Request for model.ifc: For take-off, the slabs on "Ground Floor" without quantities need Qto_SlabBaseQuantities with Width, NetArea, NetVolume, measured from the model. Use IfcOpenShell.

First a look at what the model holds.

```python
import ifcopenshell
import ifcopenshell.util.element
import ifcopenshell.util.unit

model = ifcopenshell.open("model.ifc")
print(model.schema)
for unit_type in ("LENGTHUNIT", "AREAUNIT", "VOLUMEUNIT"):
    print(unit_type, ifcopenshell.util.unit.calculate_unit_scale(model, unit_type))
storey = next(s for s in model.by_type("IfcBuildingStorey") if s.Name == "Ground Floor")
slabs = [e for e in ifcopenshell.util.element.get_decomposition(storey) if e.is_a("IfcSlab")]
for e in sorted(slabs, key=lambda e: e.id()):
    print(e.id(), e.is_a(), e.Name, list(ifcopenshell.util.element.get_psets(e, qtos_only=True)), sep=" | ")
```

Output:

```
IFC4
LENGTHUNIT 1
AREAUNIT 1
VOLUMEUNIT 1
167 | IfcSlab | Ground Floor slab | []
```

```python
import ifcopenshell
import ifcopenshell.api.pset
import ifcopenshell.geom
import ifcopenshell.util.element
import ifcopenshell.util.shape
import ifcopenshell.util.unit

model = ifcopenshell.open("model.ifc")
unit_scale = ifcopenshell.util.unit.calculate_unit_scale(model)
area_scale = ifcopenshell.util.unit.calculate_unit_scale(model, "AREAUNIT")
volume_scale = ifcopenshell.util.unit.calculate_unit_scale(model, "VOLUMEUNIT")
settings = ifcopenshell.geom.settings()

storey = next(s for s in model.by_type("IfcBuildingStorey") if s.Name == "Ground Floor")
slabs = [e for e in ifcopenshell.util.element.get_decomposition(storey) if e.is_a("IfcSlab")]

for e in sorted(slabs, key=lambda e: e.id()):
    if ifcopenshell.util.element.get_psets(e, qtos_only=True, should_inherit=False):
        continue
    # Geometry comes back in metres, in the element's own axes.
    shape = ifcopenshell.geom.create_shape(settings, e)
    values = {
        "Width": ifcopenshell.util.shape.get_z(shape.geometry) / unit_scale,
        "NetArea": ifcopenshell.util.shape.get_footprint_area(shape.geometry) / area_scale,
        "NetVolume": ifcopenshell.util.shape.get_volume(shape.geometry) / volume_scale,
    }
    qto = ifcopenshell.api.pset.add_qto(model, product=e, name="Qto_SlabBaseQuantities")
    ifcopenshell.api.pset.edit_qto(model, qto=qto, properties=values)
    print(e.id(), {k: round(v, 3) for k, v in values.items()})

model.write("model_v2.ifc")
```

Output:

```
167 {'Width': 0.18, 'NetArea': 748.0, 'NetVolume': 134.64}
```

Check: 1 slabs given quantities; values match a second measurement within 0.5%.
